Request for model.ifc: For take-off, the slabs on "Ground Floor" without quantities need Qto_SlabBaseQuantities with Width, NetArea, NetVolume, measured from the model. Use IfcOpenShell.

First a look at what the model holds.

```python
import ifcopenshell
import ifcopenshell.util.element
import ifcopenshell.util.unit

model = ifcopenshell.open("model.ifc")
print(model.schema)
for unit_type in ("LENGTHUNIT", "AREAUNIT", "VOLUMEUNIT"):
    print(unit_type, ifcopenshell.util.unit.calculate_unit_scale(model, unit_type))
storey = next(s for s in model.by_type("IfcBuildingStorey") if s.Name == "Ground Floor")
slabs = [e for e in ifcopenshell.util.element.get_decomposition(storey) if e.is_a("IfcSlab")]
for e in sorted(slabs, key=lambda e: e.id()):
    print(e.id(), e.is_a(), e.Name, list(ifcopenshell.util.element.get_psets(e, qtos_only=True)), sep=" | ")
```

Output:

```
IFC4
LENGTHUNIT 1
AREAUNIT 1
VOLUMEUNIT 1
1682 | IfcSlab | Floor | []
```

```python
import ifcopenshell
import ifcopenshell.api.pset
import ifcopenshell.geom
import ifcopenshell.util.element
import ifcopenshell.util.shape
import ifcopenshell.util.unit

model = ifcopenshell.open("model.ifc")
unit_scale = ifcopenshell.util.unit.calculate_unit_scale(model)
area_scale = ifcopenshell.util.unit.calculate_unit_scale(model, "AREAUNIT")
volume_scale = ifcopenshell.util.unit.calculate_unit_scale(model, "VOLUMEUNIT")
settings = ifcopenshell.geom.settings()

storey = next(s for s in model.by_type("IfcBuildingStorey") if s.Name == "Ground Floor")
slabs = [e for e in ifcopenshell.util.element.get_decomposition(storey) if e.is_a("IfcSlab")]

for e in sorted(slabs, key=lambda e: e.id()):
    if ifcopenshell.util.element.get_psets(e, qtos_only=True, should_inherit=False):
        continue
    # Geometry comes back in metres, in the element's own axes.
    shape = ifcopenshell.geom.create_shape(settings, e)
    values = {
        "Width": ifcopenshell.util.shape.get_z(shape.geometry) / unit_scale,
        "NetArea": ifcopenshell.util.shape.get_footprint_area(shape.geometry) / area_scale,
        "NetVolume": ifcopenshell.util.shape.get_volume(shape.geometry) / volume_scale,
    }
    qto = ifcopenshell.api.pset.add_qto(model, product=e, name="Qto_SlabBaseQuantities")
    ifcopenshell.api.pset.edit_qto(model, qto=qto, properties=values)
    print(e.id(), {k: round(v, 3) for k, v in values.items()})

model.write("model_v2.ifc")
```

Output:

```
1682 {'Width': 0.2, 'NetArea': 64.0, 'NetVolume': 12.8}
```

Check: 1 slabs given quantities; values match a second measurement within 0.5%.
